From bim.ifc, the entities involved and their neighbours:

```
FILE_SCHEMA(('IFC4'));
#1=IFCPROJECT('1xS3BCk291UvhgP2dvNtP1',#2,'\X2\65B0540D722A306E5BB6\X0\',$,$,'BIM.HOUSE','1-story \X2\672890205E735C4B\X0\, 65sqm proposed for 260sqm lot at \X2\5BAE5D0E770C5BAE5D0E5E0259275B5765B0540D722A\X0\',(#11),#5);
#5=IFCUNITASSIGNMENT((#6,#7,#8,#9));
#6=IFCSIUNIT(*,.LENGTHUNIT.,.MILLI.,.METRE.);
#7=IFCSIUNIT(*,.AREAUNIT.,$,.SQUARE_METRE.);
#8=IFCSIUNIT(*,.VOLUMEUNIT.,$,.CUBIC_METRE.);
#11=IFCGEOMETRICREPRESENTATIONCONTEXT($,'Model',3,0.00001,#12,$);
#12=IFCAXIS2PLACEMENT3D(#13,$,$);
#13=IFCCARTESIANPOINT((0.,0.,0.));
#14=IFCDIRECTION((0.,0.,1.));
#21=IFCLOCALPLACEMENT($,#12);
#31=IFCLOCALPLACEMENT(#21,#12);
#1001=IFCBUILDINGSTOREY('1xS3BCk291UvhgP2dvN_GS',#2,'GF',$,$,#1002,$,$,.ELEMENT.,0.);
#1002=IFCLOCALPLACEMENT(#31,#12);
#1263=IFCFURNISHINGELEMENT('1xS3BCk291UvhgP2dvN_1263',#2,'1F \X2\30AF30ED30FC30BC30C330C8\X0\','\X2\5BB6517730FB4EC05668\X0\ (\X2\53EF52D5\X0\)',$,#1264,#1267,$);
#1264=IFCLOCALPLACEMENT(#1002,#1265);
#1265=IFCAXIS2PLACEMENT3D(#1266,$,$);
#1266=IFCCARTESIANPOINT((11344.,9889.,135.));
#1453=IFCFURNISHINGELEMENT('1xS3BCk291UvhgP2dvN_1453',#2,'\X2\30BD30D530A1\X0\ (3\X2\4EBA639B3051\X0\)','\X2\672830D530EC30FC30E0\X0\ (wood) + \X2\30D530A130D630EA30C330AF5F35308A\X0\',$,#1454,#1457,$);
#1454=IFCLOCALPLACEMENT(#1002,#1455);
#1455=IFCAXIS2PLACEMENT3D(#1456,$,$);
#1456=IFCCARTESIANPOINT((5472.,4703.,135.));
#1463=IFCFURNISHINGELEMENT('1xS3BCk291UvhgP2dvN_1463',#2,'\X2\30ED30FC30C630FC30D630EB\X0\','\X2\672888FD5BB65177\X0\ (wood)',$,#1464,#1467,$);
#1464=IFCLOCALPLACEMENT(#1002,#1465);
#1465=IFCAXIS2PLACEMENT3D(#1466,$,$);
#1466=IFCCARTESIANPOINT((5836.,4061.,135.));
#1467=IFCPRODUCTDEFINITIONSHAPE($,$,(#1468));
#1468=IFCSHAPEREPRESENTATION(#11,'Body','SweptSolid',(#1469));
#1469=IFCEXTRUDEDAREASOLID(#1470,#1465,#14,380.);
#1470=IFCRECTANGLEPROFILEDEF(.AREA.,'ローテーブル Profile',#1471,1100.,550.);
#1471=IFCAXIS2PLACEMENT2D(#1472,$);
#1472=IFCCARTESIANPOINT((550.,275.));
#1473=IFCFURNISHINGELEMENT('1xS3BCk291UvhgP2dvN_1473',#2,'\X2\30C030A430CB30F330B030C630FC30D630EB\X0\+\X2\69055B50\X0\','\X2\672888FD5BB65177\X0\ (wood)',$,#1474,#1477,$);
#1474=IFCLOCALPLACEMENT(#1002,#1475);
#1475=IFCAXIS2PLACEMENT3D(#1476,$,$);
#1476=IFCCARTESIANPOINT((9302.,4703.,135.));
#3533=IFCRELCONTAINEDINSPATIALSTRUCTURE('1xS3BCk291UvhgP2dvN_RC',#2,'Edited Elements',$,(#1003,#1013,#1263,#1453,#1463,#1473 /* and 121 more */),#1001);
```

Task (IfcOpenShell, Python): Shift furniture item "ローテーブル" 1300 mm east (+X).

```python
import ifcopenshell
import ifcopenshell.api.geometry
import ifcopenshell.util.placement

model = ifcopenshell.open("bim.ifc")

item = model.by_guid("1xS3BCk291UvhgP2dvN_1463")
matrix = ifcopenshell.util.placement.get_local_placement(item.ObjectPlacement)
matrix[0, 3] += 1300.0
ifcopenshell.api.geometry.edit_object_placement(model, product=item, matrix=matrix, is_si=False)

print(ifcopenshell.util.placement.get_local_placement(item.ObjectPlacement).round(3) + 0.0)

model.write("bim_updated.ifc")
```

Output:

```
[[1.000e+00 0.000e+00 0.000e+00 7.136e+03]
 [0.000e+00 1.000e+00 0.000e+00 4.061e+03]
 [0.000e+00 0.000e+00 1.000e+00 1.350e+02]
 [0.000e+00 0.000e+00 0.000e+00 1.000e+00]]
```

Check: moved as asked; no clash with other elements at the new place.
